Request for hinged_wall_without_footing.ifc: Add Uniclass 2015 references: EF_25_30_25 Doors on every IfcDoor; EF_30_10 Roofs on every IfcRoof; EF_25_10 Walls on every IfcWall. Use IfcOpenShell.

First a look at what the model holds.

```python
import ifcopenshell

model = ifcopenshell.open("hinged_wall_without_footing.ifc")
print(model.schema)
print("classifications:", [c.Name for c in model.by_type("IfcClassification")])
for ifc_class in ("IfcDoor", "IfcRoof", "IfcStair", "IfcWall", "IfcWindow"):
    print(ifc_class, len(model.by_type(ifc_class)))
```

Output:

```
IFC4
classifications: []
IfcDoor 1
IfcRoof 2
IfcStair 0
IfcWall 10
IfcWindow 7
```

```python
import ifcopenshell
import ifcopenshell.api.classification

model = ifcopenshell.open("hinged_wall_without_footing.ifc")

system = ifcopenshell.api.classification.add_classification(model, classification="Uniclass 2015")

codes = {
    "IfcDoor": ("EF_25_30_25", "Doors"),
    "IfcRoof": ("EF_30_10", "Roofs"),
    "IfcWall": ("EF_25_10", "Walls"),
}
for ifc_class, (code, name) in codes.items():
    products = model.by_type(ifc_class)
    ifcopenshell.api.classification.add_reference(
        model, products=products, classification=system, identification=code, name=name
    )
    print(code, len(products))

model.write("hinged_wall_without_footing_updated.ifc")
```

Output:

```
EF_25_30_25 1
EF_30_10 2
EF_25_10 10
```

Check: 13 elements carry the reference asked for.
